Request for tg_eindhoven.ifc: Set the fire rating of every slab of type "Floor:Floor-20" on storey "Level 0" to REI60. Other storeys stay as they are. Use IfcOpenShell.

First a look at what the model holds.

```python
import ifcopenshell
import ifcopenshell.util.element

model = ifcopenshell.open("tg_eindhoven.ifc")
print(model.schema)
storey = next(s for s in model.by_type("IfcBuildingStorey") if s.Name == "Level 0")
slabs = [e for e in ifcopenshell.util.element.get_decomposition(storey) if e.is_a("IfcSlab")]
seen = {}
for e in slabs:
    element_type = ifcopenshell.util.element.get_type(e)
    key = (element_type.Name if element_type != e and element_type else None, ifcopenshell.util.element.get_pset(e, "Pset_SlabCommon", "FireRating"))
    seen[key] = seen.get(key, 0) + 1
for (name, value), count in sorted(seen.items(), key=str):
    print(count, "x", name, "|", value)
```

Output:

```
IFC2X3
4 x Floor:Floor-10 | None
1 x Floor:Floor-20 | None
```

```python
import ifcopenshell
import ifcopenshell.api.pset
import ifcopenshell.util.element

model = ifcopenshell.open("tg_eindhoven.ifc")

storey = next(s for s in model.by_type("IfcBuildingStorey") if s.Name == "Level 0")
slabs = [e for e in ifcopenshell.util.element.get_decomposition(storey) if e.is_a("IfcSlab")]

count = 0
for e in slabs:
    element_type = ifcopenshell.util.element.get_type(e)
    if element_type in (None, e) or element_type.Name != "Floor:Floor-20":
        continue
    # add_pset returns the element's existing set when there is one.
    pset = ifcopenshell.api.pset.add_pset(model, product=e, name="Pset_SlabCommon")
    ifcopenshell.api.pset.edit_pset(model, pset=pset, properties={"FireRating": "REI60"})
    count += 1

print(count, "slabs updated")

model.write("tg_eindhoven_rev.ifc")
```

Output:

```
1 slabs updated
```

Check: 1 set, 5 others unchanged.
